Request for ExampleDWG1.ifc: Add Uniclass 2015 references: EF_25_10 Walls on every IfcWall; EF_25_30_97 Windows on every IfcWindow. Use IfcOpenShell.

First a look at what the model holds.

```python
import ifcopenshell

model = ifcopenshell.open("ExampleDWG1.ifc")
print(model.schema)
print("classifications:", [c.Name for c in model.by_type("IfcClassification")])
for ifc_class in ("IfcDoor", "IfcRoof", "IfcStair", "IfcWall", "IfcWindow"):
    print(ifc_class, len(model.by_type(ifc_class)))
```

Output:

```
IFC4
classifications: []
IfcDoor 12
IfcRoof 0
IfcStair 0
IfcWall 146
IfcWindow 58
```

```python
import ifcopenshell
import ifcopenshell.api.classification

model = ifcopenshell.open("ExampleDWG1.ifc")

system = ifcopenshell.api.classification.add_classification(model, classification="Uniclass 2015")

codes = {
    "IfcWall": ("EF_25_10", "Walls"),
    "IfcWindow": ("EF_25_30_97", "Windows"),
}
for ifc_class, (code, name) in codes.items():
    products = model.by_type(ifc_class)
    ifcopenshell.api.classification.add_reference(
        model, products=products, classification=system, identification=code, name=name
    )
    print(code, len(products))

model.write("ExampleDWG1-out.ifc")
```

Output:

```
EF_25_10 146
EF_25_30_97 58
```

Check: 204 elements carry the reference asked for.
